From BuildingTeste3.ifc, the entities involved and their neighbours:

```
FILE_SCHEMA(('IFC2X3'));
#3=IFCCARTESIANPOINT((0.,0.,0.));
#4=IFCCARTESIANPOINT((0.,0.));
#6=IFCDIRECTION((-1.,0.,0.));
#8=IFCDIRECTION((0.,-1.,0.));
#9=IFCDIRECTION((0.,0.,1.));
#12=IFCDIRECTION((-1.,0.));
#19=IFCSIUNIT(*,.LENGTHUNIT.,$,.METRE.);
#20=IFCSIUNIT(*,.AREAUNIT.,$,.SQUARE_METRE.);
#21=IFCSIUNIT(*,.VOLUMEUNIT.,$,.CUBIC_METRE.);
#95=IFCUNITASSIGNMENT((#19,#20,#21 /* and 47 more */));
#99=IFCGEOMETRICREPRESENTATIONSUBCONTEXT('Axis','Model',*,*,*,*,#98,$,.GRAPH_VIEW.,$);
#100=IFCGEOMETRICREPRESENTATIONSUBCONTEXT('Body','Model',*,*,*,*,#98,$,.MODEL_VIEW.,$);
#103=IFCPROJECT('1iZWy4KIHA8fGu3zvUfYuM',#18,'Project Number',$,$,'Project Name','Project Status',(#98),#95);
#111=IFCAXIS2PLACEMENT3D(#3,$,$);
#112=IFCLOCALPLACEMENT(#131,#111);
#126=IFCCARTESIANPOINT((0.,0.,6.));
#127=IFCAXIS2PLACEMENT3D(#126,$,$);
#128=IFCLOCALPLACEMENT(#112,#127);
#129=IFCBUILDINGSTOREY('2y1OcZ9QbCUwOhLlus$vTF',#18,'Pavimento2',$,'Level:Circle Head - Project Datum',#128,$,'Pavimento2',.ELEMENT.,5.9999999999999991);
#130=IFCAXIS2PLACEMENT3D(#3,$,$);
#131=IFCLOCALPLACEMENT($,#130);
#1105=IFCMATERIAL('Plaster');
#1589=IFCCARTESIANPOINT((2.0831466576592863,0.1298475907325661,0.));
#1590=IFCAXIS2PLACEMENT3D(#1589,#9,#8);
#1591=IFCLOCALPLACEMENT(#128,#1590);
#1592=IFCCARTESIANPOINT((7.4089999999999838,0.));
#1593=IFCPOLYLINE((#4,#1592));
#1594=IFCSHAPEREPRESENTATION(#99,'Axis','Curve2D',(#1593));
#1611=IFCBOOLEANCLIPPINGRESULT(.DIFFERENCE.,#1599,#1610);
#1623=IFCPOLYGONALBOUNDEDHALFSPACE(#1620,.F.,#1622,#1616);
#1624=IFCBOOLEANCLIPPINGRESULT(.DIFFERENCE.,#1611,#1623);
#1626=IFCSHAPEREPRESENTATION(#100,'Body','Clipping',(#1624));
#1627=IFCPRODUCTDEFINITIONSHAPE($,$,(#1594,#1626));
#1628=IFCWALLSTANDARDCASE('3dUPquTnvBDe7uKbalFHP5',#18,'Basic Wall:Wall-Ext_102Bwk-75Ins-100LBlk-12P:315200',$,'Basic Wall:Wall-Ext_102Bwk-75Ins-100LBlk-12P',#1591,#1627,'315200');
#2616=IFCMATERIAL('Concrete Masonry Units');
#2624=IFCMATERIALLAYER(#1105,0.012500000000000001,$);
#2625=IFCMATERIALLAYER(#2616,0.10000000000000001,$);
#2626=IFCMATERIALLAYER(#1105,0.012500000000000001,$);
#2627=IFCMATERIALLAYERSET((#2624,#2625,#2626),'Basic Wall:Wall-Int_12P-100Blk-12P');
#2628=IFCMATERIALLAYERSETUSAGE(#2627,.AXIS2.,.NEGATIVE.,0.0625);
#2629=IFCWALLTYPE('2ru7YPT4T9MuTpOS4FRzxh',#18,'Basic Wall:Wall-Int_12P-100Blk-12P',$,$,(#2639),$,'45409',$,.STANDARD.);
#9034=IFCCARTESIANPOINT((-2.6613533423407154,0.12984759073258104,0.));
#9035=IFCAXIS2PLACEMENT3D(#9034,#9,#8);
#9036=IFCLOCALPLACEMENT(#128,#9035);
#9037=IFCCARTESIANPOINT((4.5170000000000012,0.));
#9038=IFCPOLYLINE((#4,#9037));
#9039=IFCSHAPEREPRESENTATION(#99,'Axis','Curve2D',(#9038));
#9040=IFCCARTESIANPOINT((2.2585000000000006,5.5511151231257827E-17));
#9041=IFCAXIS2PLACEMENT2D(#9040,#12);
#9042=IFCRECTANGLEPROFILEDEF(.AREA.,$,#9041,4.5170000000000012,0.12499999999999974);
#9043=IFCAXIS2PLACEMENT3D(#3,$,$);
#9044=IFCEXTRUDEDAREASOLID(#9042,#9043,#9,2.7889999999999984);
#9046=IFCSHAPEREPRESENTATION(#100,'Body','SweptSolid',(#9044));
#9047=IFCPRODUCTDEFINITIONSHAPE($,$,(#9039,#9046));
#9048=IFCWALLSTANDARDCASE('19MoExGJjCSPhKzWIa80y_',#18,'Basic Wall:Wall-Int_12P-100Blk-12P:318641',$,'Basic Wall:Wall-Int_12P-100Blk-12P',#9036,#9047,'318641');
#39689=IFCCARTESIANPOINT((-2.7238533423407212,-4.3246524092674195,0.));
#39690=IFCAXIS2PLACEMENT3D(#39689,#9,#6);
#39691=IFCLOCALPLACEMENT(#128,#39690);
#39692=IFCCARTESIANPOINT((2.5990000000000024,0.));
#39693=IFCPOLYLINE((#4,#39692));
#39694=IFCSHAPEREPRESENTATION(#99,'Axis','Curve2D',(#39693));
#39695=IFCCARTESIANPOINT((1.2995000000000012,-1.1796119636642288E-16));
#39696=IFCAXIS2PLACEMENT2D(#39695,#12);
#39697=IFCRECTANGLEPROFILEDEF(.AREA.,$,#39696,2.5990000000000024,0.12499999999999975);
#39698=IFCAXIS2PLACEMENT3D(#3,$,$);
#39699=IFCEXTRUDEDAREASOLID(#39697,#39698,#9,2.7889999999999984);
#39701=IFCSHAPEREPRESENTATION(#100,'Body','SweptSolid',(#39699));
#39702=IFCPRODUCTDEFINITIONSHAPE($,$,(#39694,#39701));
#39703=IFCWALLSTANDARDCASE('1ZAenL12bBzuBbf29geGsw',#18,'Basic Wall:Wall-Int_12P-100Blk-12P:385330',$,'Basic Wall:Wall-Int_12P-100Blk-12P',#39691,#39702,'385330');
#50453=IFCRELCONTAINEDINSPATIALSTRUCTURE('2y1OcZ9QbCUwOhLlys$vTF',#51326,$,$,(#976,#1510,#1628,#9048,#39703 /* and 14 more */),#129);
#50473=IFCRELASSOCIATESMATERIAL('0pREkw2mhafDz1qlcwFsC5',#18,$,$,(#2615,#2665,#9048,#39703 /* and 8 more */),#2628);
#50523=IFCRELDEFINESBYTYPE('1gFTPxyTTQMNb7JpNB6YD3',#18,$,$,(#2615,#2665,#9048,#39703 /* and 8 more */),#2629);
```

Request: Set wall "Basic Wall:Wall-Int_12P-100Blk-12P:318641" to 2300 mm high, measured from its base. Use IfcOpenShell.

```python
import ifcopenshell
import ifcopenshell.geom
import ifcopenshell.util.representation
import ifcopenshell.util.shape
import ifcopenshell.util.unit

model = ifcopenshell.open("BuildingTeste3.ifc")
unit_scale = ifcopenshell.util.unit.calculate_unit_scale(model)
settings = ifcopenshell.geom.settings()


def volume(element):
    """Net volume in cubic metres, openings subtracted."""
    shape = ifcopenshell.geom.create_shape(settings, element)
    return ifcopenshell.util.shape.get_volume(shape.geometry)


wall = model.by_id(9048)
before = volume(wall)

body = ifcopenshell.util.representation.get_representation(wall, "Model", "Body")
solid = body.Items[0]
old_height = solid.Depth
solid.Depth = 2.3 / unit_scale
after = volume(wall)

print(f"height {old_height:g} -> {solid.Depth:g}, volume {before:.3f} -> {after:.3f} m3")

model.write("BuildingTeste3_edited.ifc")
```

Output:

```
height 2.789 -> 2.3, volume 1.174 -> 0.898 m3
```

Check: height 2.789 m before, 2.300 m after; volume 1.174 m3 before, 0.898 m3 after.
